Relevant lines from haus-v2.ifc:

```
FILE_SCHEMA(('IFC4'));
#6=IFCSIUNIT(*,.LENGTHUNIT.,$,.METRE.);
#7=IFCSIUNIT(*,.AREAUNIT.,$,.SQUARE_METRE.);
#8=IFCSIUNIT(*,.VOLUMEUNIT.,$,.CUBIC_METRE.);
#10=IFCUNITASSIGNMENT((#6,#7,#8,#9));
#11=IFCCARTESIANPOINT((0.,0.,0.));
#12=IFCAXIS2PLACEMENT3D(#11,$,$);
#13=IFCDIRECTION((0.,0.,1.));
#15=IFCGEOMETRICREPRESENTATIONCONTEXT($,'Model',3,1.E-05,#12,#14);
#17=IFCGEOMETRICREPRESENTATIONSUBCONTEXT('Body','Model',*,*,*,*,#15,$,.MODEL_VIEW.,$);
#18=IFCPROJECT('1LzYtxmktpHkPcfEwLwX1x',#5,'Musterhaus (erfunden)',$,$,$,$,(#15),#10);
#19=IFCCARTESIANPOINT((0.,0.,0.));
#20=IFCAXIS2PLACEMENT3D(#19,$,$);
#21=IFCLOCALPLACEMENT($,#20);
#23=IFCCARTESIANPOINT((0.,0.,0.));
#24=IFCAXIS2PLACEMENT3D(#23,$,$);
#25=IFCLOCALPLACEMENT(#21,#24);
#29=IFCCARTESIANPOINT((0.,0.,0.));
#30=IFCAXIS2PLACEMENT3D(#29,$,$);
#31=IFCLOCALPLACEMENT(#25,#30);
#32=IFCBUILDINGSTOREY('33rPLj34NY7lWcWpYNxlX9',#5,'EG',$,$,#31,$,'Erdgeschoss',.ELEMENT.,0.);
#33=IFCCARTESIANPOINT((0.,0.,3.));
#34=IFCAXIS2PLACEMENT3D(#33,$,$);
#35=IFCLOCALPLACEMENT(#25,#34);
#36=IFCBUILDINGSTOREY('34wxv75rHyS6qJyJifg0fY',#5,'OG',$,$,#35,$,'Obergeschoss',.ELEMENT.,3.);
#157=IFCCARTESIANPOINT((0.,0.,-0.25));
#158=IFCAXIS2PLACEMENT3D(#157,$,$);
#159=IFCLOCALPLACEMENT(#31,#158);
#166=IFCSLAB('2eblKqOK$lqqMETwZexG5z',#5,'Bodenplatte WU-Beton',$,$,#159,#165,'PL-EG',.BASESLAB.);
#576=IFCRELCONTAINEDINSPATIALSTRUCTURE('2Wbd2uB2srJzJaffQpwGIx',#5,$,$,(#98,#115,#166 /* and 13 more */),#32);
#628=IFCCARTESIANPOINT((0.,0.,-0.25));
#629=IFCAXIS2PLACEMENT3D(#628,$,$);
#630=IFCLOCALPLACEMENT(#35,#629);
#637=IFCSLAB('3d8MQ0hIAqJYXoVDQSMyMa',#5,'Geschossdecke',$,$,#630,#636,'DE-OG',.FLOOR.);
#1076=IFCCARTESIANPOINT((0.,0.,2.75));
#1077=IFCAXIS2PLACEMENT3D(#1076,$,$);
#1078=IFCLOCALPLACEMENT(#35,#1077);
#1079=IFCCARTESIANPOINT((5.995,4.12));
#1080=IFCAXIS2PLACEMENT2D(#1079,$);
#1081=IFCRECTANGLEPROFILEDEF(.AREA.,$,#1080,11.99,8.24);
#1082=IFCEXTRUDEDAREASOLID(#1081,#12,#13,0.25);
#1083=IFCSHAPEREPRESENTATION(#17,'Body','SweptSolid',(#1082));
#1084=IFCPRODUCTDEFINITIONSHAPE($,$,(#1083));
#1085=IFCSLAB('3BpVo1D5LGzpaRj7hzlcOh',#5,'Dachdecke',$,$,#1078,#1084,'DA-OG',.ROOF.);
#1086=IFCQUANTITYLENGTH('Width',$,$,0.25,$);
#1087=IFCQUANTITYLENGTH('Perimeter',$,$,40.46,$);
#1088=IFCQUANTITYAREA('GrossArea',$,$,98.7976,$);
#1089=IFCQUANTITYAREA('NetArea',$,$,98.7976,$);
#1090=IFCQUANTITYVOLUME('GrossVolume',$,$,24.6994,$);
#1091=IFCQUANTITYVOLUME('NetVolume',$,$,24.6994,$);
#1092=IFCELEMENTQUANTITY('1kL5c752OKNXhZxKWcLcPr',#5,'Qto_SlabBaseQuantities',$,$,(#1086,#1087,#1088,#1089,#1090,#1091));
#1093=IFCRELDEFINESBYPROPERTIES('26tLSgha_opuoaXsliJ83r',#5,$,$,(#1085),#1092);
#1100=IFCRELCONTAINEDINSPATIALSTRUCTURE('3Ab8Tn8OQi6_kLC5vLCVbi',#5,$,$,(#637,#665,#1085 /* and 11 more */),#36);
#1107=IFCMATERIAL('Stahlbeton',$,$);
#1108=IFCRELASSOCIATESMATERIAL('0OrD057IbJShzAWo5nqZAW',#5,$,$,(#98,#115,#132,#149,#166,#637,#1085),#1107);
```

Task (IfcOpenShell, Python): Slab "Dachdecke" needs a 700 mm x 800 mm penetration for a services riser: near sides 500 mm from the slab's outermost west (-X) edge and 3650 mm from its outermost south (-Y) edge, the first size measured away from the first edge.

```python
import numpy as np
import ifcopenshell
import ifcopenshell.api.feature
import ifcopenshell.api.geometry
import ifcopenshell.api.pset
import ifcopenshell.api.root
import ifcopenshell.geom
import ifcopenshell.util.element
import ifcopenshell.util.placement
import ifcopenshell.util.representation
import ifcopenshell.util.shape
import ifcopenshell.util.unit

model = ifcopenshell.open("haus-v2.ifc")
unit_scale = ifcopenshell.util.unit.calculate_unit_scale(model)
area_scale = ifcopenshell.util.unit.calculate_unit_scale(model, "AREAUNIT")
volume_scale = ifcopenshell.util.unit.calculate_unit_scale(model, "VOLUMEUNIT")
settings = ifcopenshell.geom.settings()


def volume(element):
    """Net volume in cubic metres, openings subtracted."""
    shape = ifcopenshell.geom.create_shape(settings, element)
    return ifcopenshell.util.shape.get_volume(shape.geometry)


slab = model.by_id(1085)
before = volume(slab)

# Extent in the slab's own axes, in metres. The edges named are its -X and -Y sides.
slab_shape = ifcopenshell.geom.create_shape(settings, slab)
vertices = ifcopenshell.util.shape.get_vertices(slab_shape.geometry)
x_min, y_min, bottom = vertices.min(axis=0)
top = vertices[:, 2].max()

opening = ifcopenshell.api.root.create_entity(model, ifc_class="IfcOpeningElement", name="Services riser opening", predefined_type="OPENING")
context = ifcopenshell.util.representation.get_context(model, "Model", "Body", "MODEL_VIEW")
width, depth = 0.7, 0.8
outline = [(0.0, 0.0), (width, 0.0), (width, depth), (0.0, depth), (0.0, 0.0)]
# Overshoot both faces by 50 mm so the cut is clean.
shape = ifcopenshell.api.geometry.add_slab_representation(
    model, context=context, depth=top - bottom + 0.1, polyline=outline
)
ifcopenshell.api.geometry.assign_representation(model, product=opening, representation=shape)

matrix = ifcopenshell.util.placement.get_local_placement(slab.ObjectPlacement)
matrix[:, 3] = matrix @ np.append(np.array([x_min + 0.5, y_min + 3.65, bottom - 0.05]) / unit_scale, 1.0)
ifcopenshell.api.geometry.edit_object_placement(model, product=opening, matrix=matrix, is_si=False)
ifcopenshell.api.feature.add_feature(model, feature=opening, element=slab)

after = volume(slab)

# Update the slab's stored quantities.
qto = model.by_id(ifcopenshell.util.element.get_pset(slab, "Qto_SlabBaseQuantities", should_inherit=False)["id"])
ifcopenshell.api.pset.edit_qto(model, qto=qto, properties={
    "NetArea": after / (top - bottom) / area_scale,
    "NetVolume": after / volume_scale,
})

print(f"slab volume {before:.3f} -> {after:.3f} m3")

model.write("haus-v2_edited.ifc")
```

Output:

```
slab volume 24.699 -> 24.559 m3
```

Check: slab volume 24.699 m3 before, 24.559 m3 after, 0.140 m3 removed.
